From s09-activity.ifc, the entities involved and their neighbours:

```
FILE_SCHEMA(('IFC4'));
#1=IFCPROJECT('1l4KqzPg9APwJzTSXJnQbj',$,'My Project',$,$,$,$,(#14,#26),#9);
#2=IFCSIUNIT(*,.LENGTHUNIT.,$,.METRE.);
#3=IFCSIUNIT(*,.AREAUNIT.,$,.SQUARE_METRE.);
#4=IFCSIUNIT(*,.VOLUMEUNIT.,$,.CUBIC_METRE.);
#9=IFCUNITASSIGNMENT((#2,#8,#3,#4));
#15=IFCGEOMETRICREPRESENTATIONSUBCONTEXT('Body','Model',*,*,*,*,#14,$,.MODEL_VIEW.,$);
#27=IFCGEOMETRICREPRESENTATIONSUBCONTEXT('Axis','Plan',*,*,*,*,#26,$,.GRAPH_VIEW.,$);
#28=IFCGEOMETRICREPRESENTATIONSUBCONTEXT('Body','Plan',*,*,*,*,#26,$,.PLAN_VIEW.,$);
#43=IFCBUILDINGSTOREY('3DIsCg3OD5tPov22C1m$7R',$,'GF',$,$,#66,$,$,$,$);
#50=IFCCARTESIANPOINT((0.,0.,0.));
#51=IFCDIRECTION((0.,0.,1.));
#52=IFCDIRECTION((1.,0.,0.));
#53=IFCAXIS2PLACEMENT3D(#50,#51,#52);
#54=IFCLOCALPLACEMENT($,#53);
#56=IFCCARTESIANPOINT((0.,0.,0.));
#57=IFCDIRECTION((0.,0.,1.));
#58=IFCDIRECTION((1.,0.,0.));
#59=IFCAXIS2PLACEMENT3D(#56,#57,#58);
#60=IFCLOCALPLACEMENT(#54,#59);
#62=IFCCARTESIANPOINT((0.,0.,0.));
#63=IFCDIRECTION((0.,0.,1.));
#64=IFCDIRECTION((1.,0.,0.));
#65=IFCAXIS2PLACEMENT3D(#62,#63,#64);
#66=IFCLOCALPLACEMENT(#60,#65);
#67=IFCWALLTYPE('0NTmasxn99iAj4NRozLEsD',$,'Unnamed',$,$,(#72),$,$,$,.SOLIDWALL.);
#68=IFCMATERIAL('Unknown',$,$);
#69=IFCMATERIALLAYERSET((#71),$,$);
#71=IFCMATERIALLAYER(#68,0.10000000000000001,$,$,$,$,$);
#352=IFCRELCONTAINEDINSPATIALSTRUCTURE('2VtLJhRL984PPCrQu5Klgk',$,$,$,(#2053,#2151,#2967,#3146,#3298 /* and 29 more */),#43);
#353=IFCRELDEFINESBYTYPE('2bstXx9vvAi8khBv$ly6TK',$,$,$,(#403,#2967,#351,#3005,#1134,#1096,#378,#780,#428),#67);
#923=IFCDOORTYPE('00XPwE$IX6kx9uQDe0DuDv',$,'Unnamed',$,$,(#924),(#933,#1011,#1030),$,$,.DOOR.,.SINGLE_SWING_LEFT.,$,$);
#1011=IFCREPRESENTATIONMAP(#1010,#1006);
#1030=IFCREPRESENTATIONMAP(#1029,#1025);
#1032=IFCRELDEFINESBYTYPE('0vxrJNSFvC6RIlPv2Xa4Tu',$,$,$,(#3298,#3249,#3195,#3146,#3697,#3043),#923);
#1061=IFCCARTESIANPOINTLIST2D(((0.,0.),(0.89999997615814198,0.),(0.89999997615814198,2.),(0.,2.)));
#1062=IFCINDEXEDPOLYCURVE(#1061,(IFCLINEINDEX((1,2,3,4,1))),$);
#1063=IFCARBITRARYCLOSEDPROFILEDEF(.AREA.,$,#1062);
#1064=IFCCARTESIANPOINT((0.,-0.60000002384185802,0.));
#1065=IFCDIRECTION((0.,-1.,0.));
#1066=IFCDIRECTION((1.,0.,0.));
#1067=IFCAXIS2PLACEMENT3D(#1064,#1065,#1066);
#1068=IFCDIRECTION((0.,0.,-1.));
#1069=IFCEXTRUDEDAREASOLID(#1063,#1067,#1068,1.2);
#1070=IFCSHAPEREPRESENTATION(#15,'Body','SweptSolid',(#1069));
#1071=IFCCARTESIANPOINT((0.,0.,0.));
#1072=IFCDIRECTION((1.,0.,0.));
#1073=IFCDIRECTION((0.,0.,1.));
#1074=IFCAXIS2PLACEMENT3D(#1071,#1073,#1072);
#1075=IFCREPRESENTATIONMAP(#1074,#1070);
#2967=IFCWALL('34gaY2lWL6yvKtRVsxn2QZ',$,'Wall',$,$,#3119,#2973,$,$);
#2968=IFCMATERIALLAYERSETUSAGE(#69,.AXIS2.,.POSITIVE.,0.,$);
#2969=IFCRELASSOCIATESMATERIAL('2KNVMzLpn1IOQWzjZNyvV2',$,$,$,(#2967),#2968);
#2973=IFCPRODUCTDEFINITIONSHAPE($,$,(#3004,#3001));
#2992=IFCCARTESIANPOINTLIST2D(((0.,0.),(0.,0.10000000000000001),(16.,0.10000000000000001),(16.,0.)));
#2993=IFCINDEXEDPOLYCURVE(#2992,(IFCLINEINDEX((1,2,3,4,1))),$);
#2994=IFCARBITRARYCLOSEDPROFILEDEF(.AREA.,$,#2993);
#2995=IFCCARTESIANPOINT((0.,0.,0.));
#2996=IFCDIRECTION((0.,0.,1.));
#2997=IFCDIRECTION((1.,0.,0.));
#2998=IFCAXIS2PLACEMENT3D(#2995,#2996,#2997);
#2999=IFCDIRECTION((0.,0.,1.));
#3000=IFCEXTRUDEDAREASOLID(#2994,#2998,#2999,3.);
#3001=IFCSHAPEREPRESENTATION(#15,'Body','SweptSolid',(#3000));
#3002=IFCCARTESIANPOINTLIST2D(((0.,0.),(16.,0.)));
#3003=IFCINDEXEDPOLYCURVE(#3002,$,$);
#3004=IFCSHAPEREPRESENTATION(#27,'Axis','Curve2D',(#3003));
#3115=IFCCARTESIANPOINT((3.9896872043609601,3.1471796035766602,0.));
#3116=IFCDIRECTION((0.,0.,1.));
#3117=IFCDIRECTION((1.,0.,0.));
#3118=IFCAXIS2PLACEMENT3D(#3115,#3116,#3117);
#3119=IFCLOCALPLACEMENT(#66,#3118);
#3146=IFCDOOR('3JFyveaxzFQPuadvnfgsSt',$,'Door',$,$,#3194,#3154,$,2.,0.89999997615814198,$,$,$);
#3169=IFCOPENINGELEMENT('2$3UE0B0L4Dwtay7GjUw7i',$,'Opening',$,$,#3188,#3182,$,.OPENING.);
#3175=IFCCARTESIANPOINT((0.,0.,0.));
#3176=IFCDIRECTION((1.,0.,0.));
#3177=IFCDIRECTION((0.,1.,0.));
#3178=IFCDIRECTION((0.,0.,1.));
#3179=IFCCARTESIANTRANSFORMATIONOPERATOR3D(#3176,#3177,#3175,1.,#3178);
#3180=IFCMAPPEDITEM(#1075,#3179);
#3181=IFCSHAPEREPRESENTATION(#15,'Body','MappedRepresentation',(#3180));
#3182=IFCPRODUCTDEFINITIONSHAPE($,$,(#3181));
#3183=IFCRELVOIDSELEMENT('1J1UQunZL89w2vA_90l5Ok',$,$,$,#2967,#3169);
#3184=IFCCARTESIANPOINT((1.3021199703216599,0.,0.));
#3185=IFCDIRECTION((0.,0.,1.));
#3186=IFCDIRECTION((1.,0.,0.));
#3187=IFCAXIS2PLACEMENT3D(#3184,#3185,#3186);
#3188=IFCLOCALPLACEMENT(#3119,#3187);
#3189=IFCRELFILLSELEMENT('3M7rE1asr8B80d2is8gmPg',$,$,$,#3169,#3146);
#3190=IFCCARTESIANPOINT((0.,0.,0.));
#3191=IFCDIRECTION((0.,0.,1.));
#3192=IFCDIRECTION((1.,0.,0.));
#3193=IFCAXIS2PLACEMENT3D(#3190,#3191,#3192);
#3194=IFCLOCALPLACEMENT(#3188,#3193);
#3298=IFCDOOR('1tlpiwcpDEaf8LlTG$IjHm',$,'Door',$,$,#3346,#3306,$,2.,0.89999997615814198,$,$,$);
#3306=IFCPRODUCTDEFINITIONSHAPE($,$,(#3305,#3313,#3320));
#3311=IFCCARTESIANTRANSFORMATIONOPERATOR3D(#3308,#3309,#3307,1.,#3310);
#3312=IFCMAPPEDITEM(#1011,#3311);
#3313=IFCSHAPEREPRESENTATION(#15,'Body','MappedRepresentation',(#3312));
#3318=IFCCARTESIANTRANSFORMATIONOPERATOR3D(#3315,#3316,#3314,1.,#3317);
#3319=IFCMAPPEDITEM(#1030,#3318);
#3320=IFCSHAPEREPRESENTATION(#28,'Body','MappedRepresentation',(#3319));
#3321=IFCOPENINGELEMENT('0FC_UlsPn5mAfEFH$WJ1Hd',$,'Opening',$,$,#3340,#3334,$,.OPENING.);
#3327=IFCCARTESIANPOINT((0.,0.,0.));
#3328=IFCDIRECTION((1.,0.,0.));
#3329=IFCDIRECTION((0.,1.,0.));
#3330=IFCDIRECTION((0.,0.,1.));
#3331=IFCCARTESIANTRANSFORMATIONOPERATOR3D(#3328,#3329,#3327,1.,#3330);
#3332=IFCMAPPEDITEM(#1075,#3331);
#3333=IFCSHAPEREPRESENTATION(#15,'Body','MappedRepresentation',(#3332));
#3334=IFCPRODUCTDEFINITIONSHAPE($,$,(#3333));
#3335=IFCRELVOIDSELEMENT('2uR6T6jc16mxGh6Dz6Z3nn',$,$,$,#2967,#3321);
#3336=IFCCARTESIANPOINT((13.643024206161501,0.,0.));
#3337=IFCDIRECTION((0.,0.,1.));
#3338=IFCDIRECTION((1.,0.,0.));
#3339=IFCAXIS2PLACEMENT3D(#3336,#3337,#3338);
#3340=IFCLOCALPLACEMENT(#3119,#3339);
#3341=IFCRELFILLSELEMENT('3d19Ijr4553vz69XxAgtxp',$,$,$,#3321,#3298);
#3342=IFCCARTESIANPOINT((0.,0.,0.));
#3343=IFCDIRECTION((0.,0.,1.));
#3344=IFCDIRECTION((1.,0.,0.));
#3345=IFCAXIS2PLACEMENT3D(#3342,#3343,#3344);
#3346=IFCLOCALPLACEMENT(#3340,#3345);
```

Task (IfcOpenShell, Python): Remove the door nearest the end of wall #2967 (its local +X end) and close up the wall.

```python
import ifcopenshell
import ifcopenshell.api.feature
import ifcopenshell.api.root
import ifcopenshell.geom
import ifcopenshell.util.shape

model = ifcopenshell.open("s09-activity.ifc")
settings = ifcopenshell.geom.settings()


def volume(element):
    """Net volume in cubic metres, openings subtracted."""
    shape = ifcopenshell.geom.create_shape(settings, element)
    return ifcopenshell.util.shape.get_volume(shape.geometry)


door = model.by_guid("1tlpiwcpDEaf8LlTG$IjHm")
opening = door.FillsVoids[0].RelatingOpeningElement
wall = opening.VoidsElements[0].RelatingBuildingElement
before = volume(wall)

ifcopenshell.api.root.remove_product(model, product=door)
ifcopenshell.api.feature.remove_feature(model, feature=opening)

after = volume(wall)

print(f"wall volume {before:.3f} -> {after:.3f} m3")

model.write("s09-activity-out.ifc")
```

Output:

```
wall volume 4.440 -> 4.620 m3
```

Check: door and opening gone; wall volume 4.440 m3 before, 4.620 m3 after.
